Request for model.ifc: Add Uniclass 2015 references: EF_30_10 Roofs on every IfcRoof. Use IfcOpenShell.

First a look at what the model holds.

```python
import ifcopenshell

model = ifcopenshell.open("model.ifc")
print(model.schema)
print("classifications:", [c.Name for c in model.by_type("IfcClassification")])
for ifc_class in ("IfcDoor", "IfcRoof", "IfcStair", "IfcWall", "IfcWindow"):
    print(ifc_class, len(model.by_type(ifc_class)))
```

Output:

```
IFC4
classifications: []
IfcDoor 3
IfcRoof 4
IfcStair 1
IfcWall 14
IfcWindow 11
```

```python
import ifcopenshell
import ifcopenshell.api.classification

model = ifcopenshell.open("model.ifc")

system = ifcopenshell.api.classification.add_classification(model, classification="Uniclass 2015")

codes = {
    "IfcRoof": ("EF_30_10", "Roofs"),
}
for ifc_class, (code, name) in codes.items():
    products = model.by_type(ifc_class)
    ifcopenshell.api.classification.add_reference(
        model, products=products, classification=system, identification=code, name=name
    )
    print(code, len(products))

model.write("model_edited.ifc")
```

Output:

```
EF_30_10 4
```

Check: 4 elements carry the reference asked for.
